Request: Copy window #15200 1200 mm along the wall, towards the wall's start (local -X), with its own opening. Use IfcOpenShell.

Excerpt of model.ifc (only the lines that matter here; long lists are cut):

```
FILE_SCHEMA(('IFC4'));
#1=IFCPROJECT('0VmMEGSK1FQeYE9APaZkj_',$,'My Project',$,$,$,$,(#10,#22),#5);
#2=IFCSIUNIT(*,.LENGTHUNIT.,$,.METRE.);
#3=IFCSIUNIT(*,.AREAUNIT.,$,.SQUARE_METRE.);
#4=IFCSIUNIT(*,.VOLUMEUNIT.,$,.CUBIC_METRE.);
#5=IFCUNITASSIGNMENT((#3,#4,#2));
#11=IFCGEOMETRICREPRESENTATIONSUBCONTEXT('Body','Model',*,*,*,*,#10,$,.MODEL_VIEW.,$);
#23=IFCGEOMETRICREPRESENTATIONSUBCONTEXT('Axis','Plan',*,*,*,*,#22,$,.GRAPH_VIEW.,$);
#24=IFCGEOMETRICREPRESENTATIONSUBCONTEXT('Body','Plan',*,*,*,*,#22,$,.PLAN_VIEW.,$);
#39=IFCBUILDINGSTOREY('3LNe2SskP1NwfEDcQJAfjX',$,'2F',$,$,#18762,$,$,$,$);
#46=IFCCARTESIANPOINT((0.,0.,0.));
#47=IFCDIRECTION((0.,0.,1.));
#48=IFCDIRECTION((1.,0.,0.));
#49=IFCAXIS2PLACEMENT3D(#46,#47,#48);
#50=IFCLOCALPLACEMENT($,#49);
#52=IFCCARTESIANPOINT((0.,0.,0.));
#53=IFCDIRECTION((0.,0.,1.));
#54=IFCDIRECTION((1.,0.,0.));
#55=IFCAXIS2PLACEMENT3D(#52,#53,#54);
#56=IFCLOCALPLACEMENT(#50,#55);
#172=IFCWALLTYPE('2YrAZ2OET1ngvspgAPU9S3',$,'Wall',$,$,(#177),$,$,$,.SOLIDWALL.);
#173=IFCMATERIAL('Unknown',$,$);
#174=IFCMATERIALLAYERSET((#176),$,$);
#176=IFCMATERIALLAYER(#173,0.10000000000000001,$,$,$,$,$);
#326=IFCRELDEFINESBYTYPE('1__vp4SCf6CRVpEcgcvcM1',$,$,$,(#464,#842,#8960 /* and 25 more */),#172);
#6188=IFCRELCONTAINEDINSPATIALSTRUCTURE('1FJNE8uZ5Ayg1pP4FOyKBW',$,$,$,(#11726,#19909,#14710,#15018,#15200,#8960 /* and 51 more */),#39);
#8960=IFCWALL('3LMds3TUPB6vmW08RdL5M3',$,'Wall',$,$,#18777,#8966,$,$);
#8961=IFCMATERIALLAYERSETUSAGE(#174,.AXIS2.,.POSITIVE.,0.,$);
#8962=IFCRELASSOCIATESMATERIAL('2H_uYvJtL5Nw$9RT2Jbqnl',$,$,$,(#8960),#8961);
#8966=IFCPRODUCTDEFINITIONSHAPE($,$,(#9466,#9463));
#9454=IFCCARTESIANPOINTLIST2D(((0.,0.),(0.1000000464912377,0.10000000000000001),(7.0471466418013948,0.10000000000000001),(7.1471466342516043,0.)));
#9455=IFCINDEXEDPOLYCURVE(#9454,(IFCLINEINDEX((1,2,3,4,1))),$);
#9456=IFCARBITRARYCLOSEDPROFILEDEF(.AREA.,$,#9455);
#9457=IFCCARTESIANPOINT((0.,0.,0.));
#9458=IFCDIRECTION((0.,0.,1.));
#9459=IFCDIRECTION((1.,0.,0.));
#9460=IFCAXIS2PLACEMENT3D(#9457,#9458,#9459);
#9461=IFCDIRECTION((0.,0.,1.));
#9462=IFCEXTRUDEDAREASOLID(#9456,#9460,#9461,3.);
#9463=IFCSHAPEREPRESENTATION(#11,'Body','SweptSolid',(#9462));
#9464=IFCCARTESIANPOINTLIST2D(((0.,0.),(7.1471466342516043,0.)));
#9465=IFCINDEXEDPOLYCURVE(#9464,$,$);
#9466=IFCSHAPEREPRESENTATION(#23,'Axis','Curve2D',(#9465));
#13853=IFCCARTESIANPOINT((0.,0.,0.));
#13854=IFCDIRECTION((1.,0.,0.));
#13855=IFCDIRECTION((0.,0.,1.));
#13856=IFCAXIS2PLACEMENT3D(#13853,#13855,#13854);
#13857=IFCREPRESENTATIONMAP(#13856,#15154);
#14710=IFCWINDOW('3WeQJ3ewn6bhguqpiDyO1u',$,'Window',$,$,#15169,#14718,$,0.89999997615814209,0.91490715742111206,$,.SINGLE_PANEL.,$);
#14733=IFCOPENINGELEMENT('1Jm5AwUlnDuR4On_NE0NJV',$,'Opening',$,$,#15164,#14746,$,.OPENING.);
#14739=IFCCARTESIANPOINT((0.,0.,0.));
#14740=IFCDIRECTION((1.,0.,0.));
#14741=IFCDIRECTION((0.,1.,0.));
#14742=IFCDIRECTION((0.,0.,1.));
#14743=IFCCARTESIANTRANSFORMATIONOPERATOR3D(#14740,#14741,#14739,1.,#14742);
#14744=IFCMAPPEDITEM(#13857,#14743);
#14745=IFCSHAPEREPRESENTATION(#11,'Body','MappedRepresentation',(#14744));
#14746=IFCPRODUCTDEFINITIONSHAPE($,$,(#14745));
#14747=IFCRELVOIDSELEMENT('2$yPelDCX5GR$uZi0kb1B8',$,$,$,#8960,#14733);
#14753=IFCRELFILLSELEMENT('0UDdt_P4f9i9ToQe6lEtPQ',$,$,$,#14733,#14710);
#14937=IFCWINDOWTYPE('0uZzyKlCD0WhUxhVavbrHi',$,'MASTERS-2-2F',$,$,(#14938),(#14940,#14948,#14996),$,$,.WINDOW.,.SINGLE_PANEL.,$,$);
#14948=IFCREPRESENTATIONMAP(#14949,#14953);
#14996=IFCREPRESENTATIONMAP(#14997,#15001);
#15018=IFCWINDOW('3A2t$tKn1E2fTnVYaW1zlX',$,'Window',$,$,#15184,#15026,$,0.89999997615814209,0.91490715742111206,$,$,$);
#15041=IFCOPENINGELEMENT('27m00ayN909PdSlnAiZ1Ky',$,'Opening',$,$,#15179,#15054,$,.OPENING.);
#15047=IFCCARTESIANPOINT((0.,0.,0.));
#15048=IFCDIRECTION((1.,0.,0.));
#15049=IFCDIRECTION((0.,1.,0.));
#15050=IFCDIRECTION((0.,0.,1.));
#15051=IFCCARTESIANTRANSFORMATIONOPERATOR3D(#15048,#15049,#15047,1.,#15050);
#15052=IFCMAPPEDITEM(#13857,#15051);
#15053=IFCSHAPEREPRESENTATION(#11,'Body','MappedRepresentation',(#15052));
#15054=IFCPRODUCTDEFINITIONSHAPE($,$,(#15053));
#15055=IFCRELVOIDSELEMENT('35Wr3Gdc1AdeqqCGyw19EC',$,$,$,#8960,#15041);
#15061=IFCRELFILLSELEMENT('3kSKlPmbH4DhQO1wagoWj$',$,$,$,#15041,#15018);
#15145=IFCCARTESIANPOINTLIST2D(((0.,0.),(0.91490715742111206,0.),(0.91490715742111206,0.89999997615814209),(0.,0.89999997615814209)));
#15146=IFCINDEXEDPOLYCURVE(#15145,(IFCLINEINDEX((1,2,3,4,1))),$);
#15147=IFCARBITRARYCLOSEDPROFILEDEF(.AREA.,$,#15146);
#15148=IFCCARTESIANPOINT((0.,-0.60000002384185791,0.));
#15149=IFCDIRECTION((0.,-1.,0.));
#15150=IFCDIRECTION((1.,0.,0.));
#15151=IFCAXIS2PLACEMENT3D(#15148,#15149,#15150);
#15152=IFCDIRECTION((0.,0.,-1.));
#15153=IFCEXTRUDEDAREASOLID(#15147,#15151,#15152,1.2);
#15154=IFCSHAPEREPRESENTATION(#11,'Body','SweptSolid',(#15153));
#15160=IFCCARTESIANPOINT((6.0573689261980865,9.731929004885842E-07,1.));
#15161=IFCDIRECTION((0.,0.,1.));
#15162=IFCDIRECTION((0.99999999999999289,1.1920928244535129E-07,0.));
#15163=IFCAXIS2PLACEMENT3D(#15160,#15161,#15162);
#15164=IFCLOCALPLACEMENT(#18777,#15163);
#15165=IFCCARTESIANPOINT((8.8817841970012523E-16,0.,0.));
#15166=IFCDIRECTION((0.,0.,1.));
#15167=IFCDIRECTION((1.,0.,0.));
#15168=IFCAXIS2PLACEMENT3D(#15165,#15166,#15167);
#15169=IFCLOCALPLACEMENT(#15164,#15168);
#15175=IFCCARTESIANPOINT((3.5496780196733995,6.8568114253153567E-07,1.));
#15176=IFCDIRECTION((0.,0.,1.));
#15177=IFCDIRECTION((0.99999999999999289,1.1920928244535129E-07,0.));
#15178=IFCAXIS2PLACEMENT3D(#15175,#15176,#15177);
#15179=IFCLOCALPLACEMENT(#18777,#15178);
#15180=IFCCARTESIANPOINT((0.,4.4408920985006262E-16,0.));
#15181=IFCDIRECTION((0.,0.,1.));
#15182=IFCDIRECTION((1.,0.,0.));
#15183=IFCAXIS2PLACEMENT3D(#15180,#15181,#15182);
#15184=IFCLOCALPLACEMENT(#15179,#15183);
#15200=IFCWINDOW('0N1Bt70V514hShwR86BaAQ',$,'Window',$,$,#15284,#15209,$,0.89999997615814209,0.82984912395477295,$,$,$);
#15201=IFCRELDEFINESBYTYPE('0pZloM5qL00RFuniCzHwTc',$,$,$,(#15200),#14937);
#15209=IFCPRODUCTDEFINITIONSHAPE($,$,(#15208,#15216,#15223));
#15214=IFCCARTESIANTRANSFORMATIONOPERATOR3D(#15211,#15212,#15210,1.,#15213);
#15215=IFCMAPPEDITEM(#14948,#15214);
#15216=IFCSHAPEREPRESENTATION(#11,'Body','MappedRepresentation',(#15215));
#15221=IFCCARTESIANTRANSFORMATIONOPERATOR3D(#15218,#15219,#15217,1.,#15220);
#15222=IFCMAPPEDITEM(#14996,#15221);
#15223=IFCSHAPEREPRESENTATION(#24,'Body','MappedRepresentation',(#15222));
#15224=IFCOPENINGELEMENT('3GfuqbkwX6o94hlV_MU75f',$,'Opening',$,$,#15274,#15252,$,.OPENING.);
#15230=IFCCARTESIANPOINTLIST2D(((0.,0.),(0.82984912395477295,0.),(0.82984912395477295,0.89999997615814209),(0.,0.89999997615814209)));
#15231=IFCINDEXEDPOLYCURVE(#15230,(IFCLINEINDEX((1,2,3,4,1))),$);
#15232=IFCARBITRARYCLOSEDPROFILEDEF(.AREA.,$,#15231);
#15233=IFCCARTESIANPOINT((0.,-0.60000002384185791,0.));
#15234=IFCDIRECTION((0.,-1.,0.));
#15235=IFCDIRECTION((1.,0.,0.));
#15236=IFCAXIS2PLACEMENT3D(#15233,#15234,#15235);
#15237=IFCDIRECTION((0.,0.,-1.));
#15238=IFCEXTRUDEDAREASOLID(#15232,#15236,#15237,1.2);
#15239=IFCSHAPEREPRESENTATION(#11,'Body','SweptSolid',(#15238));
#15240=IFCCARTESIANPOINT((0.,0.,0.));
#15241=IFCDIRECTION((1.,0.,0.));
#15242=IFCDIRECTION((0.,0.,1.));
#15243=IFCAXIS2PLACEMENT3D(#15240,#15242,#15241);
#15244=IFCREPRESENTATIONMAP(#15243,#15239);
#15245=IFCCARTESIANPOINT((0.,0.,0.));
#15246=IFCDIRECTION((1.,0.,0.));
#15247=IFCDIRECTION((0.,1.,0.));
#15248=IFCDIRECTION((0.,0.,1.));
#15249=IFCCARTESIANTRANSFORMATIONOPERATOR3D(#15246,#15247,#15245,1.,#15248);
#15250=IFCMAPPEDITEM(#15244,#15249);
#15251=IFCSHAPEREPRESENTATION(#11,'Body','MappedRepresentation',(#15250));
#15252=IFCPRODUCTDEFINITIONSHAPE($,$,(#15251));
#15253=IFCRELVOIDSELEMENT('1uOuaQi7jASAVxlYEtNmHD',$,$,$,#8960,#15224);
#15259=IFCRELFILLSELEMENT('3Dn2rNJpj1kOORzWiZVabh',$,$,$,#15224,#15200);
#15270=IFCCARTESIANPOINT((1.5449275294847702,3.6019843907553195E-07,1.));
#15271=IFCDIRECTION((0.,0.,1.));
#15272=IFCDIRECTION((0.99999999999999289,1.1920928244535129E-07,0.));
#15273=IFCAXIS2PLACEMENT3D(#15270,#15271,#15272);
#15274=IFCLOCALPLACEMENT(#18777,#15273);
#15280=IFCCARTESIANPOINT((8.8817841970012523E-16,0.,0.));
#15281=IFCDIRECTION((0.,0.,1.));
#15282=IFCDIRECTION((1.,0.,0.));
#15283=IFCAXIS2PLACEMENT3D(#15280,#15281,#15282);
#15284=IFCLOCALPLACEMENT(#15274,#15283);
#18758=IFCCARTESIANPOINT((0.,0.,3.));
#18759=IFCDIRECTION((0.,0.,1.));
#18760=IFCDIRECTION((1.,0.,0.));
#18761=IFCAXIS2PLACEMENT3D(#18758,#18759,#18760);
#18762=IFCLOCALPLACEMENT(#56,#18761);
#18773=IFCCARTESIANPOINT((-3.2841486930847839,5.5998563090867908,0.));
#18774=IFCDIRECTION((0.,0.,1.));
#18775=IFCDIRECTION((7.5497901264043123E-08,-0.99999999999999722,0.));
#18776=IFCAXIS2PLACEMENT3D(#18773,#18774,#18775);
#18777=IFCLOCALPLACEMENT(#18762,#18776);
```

```python
import ifcopenshell
import ifcopenshell.api.feature
import ifcopenshell.api.geometry
import ifcopenshell.api.root
import ifcopenshell.geom
import ifcopenshell.util.element
import ifcopenshell.util.placement
import ifcopenshell.util.shape
import ifcopenshell.util.unit

model = ifcopenshell.open("model.ifc")
unit_scale = ifcopenshell.util.unit.calculate_unit_scale(model)
settings = ifcopenshell.geom.settings()


def volume(element):
    """Net volume in cubic metres, openings subtracted."""
    shape = ifcopenshell.geom.create_shape(settings, element)
    return ifcopenshell.util.shape.get_volume(shape.geometry)


window = model.by_guid("0N1Bt70V514hShwR86BaAQ")
opening = window.FillsVoids[0].RelatingOpeningElement
wall = opening.VoidsElements[0].RelatingBuildingElement
before = volume(wall)
shift = ifcopenshell.util.placement.get_local_placement(wall.ObjectPlacement)[:3, 0] * -1.2 / unit_scale

# copy_class copies the void relationship, type, container and properties, but no geometry.
new_opening = ifcopenshell.api.root.copy_class(model, product=opening)
new_opening.Representation = ifcopenshell.util.element.copy_deep(
    model, opening.Representation, exclude=["IfcGeometricRepresentationContext", "IfcRepresentationMap"]
)
new_window = ifcopenshell.api.root.copy_class(model, product=window)
new_window.Representation = ifcopenshell.util.element.copy_deep(
    model, window.Representation, exclude=["IfcGeometricRepresentationContext", "IfcRepresentationMap"]
)
ifcopenshell.api.feature.add_filling(model, opening=new_opening, element=new_window)

for old, new in ((opening, new_opening), (window, new_window)):
    matrix = ifcopenshell.util.placement.get_local_placement(old.ObjectPlacement)
    matrix[:3, 3] += shift
    ifcopenshell.api.geometry.edit_object_placement(model, product=new, matrix=matrix, is_si=False)

after = volume(wall)

print(f"wall volume {before:.3f} -> {after:.3f} m3")

model.write("model_rev.ifc")
```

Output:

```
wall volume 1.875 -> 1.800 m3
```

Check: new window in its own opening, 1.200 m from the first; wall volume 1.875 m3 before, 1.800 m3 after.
